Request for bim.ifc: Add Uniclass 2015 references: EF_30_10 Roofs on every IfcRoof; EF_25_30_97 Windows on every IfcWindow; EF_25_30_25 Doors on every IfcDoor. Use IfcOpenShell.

First a look at what the model holds.

```python
import ifcopenshell

model = ifcopenshell.open("bim.ifc")
print(model.schema)
print("classifications:", [c.Name for c in model.by_type("IfcClassification")])
for ifc_class in ("IfcDoor", "IfcRoof", "IfcStair", "IfcWall", "IfcWindow"):
    print(ifc_class, len(model.by_type(ifc_class)))
```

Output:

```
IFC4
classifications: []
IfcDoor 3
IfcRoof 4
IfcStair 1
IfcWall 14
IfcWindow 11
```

```python
import ifcopenshell
import ifcopenshell.api.classification

model = ifcopenshell.open("bim.ifc")

system = ifcopenshell.api.classification.add_classification(model, classification="Uniclass 2015")

codes = {
    "IfcRoof": ("EF_30_10", "Roofs"),
    "IfcWindow": ("EF_25_30_97", "Windows"),
    "IfcDoor": ("EF_25_30_25", "Doors"),
}
for ifc_class, (code, name) in codes.items():
    products = model.by_type(ifc_class)
    ifcopenshell.api.classification.add_reference(
        model, products=products, classification=system, identification=code, name=name
    )
    print(code, len(products))

model.write("bim_rev.ifc")
```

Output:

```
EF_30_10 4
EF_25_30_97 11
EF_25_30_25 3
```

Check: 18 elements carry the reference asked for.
